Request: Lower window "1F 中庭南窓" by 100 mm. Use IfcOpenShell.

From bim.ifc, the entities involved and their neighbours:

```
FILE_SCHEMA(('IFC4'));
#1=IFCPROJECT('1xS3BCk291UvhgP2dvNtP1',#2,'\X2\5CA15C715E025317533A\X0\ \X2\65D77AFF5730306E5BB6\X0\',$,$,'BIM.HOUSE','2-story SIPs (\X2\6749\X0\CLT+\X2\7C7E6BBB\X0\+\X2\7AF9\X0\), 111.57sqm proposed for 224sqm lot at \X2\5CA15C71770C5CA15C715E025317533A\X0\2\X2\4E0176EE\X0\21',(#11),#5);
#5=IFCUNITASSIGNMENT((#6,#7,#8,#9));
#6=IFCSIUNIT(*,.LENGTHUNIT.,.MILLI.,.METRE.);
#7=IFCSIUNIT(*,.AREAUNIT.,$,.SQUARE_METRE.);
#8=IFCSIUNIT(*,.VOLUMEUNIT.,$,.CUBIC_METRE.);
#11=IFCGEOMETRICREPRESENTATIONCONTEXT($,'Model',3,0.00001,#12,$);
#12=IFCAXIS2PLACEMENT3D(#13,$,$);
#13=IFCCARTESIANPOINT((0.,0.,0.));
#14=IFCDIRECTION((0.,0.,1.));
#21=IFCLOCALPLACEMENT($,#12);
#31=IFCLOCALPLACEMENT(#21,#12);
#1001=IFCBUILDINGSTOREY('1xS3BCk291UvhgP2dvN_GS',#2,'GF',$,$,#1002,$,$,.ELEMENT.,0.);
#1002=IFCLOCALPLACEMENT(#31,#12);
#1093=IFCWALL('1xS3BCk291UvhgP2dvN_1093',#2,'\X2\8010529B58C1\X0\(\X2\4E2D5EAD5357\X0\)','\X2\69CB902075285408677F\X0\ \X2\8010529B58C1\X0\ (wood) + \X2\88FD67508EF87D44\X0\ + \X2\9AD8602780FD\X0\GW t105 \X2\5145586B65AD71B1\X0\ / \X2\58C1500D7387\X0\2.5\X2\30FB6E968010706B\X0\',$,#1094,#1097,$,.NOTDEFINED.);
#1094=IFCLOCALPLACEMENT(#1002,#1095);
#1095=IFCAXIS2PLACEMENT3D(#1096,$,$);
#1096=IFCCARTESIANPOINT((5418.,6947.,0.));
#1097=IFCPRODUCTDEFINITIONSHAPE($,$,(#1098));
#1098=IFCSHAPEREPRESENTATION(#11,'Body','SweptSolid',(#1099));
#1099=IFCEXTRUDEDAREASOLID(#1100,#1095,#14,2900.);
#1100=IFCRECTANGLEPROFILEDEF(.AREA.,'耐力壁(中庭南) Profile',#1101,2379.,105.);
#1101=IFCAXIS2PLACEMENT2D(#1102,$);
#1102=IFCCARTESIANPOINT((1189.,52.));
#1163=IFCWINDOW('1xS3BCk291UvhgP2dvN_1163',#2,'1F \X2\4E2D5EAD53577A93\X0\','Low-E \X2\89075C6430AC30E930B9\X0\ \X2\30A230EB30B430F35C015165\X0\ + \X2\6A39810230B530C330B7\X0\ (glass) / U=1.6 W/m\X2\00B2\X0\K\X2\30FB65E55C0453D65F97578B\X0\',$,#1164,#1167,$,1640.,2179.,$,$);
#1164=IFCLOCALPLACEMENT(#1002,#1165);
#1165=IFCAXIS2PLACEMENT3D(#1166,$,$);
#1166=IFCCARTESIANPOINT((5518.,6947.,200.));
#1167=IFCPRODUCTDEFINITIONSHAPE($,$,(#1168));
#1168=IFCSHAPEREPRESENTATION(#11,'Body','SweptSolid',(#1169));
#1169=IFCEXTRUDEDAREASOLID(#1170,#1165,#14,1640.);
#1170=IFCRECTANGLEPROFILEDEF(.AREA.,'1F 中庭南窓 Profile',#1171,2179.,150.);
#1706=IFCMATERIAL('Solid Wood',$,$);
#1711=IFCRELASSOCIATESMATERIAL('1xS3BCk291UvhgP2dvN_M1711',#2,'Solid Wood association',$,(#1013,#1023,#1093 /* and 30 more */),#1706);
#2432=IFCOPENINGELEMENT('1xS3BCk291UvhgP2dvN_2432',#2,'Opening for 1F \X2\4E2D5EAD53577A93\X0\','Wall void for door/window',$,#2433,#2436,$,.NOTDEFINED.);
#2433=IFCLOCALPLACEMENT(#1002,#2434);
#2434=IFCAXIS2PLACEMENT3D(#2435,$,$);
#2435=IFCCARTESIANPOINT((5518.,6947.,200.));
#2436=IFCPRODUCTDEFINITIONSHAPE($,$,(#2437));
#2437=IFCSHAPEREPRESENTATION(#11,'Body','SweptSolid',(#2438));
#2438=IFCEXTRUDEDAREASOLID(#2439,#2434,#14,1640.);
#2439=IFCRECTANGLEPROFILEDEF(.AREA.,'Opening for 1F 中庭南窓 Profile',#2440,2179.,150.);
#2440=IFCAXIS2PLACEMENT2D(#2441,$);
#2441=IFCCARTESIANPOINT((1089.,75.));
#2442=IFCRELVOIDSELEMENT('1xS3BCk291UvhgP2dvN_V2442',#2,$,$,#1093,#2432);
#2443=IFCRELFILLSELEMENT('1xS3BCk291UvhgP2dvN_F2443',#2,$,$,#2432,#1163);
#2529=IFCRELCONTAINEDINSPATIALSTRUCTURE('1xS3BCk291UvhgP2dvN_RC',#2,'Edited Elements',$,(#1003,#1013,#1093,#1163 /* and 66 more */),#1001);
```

```python
import numpy as np
import ifcopenshell
import ifcopenshell.api.geometry
import ifcopenshell.util.placement
import ifcopenshell.util.unit

model = ifcopenshell.open("bim.ifc")
unit_scale = ifcopenshell.util.unit.calculate_unit_scale(model)

window = model.by_guid("1xS3BCk291UvhgP2dvN_1163")
opening = window.FillsVoids[0].RelatingOpeningElement
dz = -100.0

shift = np.array([0.0, 0.0, dz])
# The window is not placed relative to its opening, so move both.
for product in (opening, window):
    matrix = ifcopenshell.util.placement.get_local_placement(product.ObjectPlacement)
    matrix[:3, 3] += shift
    ifcopenshell.api.geometry.edit_object_placement(model, product=product, matrix=matrix, is_si=False)

print(f"moved by {dz * unit_scale:+.3f} m")

model.write("bim_edited.ifc")
```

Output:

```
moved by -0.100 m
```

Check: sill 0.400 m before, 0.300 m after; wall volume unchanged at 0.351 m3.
